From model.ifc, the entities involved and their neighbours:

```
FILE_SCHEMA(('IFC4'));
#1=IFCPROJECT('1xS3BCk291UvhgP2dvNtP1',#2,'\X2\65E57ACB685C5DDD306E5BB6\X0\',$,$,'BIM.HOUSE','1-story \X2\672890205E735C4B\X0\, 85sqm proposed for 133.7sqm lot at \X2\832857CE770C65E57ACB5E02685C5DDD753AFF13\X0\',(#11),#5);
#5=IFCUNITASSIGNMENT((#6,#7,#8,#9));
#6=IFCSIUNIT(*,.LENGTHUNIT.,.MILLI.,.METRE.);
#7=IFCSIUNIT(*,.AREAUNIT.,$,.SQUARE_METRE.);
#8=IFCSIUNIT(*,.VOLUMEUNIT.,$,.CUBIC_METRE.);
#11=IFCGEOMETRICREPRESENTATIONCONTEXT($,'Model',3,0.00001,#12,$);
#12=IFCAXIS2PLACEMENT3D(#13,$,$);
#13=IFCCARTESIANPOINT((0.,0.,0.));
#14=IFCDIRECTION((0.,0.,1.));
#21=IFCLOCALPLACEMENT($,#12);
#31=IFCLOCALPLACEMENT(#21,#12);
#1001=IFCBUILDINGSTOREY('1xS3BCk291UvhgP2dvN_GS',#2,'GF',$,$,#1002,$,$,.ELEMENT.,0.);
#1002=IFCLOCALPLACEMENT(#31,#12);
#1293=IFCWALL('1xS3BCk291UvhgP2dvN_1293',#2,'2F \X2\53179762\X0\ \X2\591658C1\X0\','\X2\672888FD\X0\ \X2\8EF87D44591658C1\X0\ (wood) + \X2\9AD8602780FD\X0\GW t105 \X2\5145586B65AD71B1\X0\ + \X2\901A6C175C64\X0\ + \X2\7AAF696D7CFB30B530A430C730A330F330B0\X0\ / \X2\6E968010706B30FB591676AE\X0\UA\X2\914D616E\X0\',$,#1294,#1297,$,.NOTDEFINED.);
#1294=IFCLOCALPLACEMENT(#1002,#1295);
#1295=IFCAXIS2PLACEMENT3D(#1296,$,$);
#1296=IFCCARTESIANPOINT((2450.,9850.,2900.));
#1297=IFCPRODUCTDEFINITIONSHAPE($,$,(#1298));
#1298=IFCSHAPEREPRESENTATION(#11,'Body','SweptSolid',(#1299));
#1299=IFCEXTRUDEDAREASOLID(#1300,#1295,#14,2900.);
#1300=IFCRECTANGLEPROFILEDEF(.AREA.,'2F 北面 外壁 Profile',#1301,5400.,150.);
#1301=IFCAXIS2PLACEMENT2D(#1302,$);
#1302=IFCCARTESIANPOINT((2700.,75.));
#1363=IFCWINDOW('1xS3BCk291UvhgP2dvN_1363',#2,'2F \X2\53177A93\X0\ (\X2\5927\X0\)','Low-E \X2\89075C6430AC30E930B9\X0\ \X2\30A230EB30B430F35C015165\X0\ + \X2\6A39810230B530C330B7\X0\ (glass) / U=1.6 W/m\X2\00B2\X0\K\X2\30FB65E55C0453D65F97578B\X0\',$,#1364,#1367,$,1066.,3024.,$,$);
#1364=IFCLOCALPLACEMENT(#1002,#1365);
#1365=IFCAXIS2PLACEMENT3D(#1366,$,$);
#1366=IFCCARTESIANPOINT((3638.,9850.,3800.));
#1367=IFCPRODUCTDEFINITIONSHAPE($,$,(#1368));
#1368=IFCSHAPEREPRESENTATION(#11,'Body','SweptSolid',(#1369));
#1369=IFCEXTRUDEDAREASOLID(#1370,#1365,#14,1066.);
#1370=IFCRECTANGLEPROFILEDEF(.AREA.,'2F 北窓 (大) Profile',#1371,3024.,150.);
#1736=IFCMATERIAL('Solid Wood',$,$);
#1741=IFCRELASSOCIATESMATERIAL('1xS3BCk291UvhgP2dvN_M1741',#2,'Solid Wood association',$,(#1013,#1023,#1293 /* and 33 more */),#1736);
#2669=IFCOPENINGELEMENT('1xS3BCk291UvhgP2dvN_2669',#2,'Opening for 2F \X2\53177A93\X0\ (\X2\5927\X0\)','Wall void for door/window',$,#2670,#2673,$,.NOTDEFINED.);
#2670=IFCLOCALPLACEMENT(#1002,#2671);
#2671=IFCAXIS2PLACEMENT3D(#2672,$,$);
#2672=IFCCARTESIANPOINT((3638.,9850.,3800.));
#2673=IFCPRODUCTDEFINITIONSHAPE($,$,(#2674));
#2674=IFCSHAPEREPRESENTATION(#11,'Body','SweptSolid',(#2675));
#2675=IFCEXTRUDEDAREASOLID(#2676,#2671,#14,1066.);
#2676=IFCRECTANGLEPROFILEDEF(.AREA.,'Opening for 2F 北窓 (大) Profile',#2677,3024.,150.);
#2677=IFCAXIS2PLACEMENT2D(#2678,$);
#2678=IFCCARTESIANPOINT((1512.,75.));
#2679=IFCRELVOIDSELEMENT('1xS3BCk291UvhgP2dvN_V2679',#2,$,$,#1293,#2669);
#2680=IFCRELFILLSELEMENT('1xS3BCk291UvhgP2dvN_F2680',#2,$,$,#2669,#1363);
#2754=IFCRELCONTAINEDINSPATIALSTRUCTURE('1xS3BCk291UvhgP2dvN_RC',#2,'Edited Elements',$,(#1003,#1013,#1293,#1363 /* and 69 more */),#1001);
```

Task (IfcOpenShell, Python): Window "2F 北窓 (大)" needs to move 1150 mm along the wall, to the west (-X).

```python
import ifcopenshell
import ifcopenshell.api.geometry
import ifcopenshell.util.placement

model = ifcopenshell.open("model.ifc")

window = model.by_guid("1xS3BCk291UvhgP2dvN_1363")
opening = window.FillsVoids[0].RelatingOpeningElement
wall = opening.VoidsElements[0].RelatingBuildingElement

wall_matrix = ifcopenshell.util.placement.get_local_placement(wall.ObjectPlacement)
shift = wall_matrix[:3, 0] * -1150.0
before = ifcopenshell.util.placement.get_local_placement(window.ObjectPlacement)[:3, 3].copy()

# The window is not placed relative to its opening, so move both.
for product in (opening, window):
    matrix = ifcopenshell.util.placement.get_local_placement(product.ObjectPlacement)
    matrix[:3, 3] += shift
    ifcopenshell.api.geometry.edit_object_placement(model, product=product, matrix=matrix, is_si=False)

after = ifcopenshell.util.placement.get_local_placement(window.ObjectPlacement)[:3, 3]
print("window moved by", (after - before).round(3) + 0.0)

model.write("model_edited.ifc")
```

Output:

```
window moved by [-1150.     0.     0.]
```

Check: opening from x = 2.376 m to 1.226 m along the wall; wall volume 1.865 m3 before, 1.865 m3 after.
